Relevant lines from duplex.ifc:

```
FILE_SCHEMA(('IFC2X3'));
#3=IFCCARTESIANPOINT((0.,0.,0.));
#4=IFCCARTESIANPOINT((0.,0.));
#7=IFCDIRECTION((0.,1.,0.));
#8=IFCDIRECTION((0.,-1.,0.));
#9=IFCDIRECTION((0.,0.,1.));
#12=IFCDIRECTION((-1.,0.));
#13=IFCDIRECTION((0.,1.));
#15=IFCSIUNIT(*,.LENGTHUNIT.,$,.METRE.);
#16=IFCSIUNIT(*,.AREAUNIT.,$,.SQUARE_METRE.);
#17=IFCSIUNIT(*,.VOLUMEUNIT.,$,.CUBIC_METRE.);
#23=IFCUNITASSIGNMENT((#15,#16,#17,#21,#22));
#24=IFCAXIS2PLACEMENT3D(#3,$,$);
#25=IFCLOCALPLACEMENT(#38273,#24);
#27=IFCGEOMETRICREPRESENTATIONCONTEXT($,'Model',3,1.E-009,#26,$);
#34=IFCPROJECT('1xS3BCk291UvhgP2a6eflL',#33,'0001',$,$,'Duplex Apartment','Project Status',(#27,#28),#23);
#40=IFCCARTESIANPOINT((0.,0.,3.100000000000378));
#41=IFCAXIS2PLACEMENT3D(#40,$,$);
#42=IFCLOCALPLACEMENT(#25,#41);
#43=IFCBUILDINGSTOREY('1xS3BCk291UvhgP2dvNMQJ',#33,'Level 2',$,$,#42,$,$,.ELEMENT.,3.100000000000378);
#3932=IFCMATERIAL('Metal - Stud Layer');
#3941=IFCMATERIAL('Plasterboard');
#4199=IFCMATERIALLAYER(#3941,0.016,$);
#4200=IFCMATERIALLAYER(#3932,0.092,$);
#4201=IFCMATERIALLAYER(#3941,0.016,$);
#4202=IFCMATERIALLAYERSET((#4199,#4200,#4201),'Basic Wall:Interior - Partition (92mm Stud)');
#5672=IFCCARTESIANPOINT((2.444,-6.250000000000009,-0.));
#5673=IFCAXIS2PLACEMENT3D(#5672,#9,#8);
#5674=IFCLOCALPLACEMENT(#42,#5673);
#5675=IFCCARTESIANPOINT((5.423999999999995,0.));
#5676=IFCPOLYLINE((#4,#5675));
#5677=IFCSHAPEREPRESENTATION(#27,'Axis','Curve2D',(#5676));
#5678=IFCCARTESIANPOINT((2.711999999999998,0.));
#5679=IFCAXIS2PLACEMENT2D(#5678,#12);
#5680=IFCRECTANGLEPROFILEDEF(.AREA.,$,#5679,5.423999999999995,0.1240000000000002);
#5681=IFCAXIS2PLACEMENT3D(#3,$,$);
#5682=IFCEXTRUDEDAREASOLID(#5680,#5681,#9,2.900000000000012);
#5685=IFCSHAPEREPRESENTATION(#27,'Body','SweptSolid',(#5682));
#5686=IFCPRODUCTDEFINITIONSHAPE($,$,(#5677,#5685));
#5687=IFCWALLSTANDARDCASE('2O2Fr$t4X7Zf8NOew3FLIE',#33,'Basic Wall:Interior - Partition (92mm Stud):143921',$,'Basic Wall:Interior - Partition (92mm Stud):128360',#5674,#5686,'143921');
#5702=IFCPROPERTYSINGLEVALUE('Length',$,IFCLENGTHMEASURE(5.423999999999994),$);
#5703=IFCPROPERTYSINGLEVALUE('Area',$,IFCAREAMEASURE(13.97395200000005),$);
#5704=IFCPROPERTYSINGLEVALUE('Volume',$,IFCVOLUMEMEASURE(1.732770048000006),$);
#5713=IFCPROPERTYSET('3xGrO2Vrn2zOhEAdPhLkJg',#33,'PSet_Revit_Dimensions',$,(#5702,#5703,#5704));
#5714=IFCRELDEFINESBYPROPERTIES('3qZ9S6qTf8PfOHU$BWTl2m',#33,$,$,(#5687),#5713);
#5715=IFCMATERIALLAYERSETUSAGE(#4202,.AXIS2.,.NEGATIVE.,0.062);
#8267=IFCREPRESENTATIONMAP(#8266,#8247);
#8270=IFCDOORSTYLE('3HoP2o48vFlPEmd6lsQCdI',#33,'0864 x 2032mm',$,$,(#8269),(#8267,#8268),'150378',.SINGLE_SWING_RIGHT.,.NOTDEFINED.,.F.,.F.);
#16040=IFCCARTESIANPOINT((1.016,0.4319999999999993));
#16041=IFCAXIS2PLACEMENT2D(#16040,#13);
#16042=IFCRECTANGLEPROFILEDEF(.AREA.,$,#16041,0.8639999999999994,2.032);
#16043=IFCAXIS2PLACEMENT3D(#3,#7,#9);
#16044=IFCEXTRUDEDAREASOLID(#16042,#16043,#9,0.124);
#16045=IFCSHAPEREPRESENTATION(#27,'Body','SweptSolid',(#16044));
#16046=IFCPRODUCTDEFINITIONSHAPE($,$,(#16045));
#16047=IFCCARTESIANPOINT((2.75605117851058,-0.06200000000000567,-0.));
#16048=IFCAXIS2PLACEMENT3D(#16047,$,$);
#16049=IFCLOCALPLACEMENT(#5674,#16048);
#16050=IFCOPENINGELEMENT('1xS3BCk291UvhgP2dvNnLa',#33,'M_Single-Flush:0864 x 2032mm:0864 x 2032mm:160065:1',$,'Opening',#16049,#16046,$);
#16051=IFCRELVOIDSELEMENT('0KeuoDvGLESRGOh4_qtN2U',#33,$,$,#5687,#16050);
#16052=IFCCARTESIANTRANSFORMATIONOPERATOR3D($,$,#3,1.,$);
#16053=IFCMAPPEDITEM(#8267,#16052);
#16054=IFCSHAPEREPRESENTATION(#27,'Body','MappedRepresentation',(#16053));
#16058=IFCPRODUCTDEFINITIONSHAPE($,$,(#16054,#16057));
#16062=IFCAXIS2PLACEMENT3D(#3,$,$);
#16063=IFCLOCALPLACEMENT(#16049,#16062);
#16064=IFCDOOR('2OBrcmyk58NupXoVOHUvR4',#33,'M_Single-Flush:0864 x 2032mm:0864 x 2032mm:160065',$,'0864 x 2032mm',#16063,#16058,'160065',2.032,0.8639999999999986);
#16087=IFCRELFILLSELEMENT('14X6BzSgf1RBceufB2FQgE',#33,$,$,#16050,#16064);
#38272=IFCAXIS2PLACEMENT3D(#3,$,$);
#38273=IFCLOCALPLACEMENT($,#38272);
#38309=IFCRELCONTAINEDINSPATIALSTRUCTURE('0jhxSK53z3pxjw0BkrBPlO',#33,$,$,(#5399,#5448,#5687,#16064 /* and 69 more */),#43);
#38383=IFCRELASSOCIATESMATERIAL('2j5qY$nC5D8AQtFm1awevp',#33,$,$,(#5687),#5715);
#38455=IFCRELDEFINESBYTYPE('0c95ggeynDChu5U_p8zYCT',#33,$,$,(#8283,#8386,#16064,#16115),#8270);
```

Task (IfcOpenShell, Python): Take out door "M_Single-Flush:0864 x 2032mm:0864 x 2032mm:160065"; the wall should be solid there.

```python
import ifcopenshell
import ifcopenshell.api.feature
import ifcopenshell.api.pset
import ifcopenshell.api.root
import ifcopenshell.geom
import ifcopenshell.util.element
import ifcopenshell.util.shape
import ifcopenshell.util.unit

model = ifcopenshell.open("duplex.ifc")
area_scale = ifcopenshell.util.unit.calculate_unit_scale(model, "AREAUNIT")
volume_scale = ifcopenshell.util.unit.calculate_unit_scale(model, "VOLUMEUNIT")
settings = ifcopenshell.geom.settings()


def volume(element):
    """Net volume in cubic metres, openings subtracted."""
    shape = ifcopenshell.geom.create_shape(settings, element)
    return ifcopenshell.util.shape.get_volume(shape.geometry)


door = model.by_guid("2OBrcmyk58NupXoVOHUvR4")
opening = door.FillsVoids[0].RelatingOpeningElement
wall = opening.VoidsElements[0].RelatingBuildingElement
before = volume(wall)

ifcopenshell.api.root.remove_product(model, product=door)
ifcopenshell.api.feature.remove_feature(model, feature=opening)

after = volume(wall)
thickness = 0.124  # wall thickness in metres

# Update the wall's stored quantities.
pset = model.by_id(ifcopenshell.util.element.get_pset(wall, "PSet_Revit_Dimensions", should_inherit=False)["id"])
ifcopenshell.api.pset.edit_pset(model, pset=pset, properties={
    "Area": model.create_entity("IfcAreaMeasure", after / thickness / area_scale),
    "Volume": model.create_entity("IfcVolumeMeasure", after / volume_scale),
})

print(f"wall volume {before:.3f} -> {after:.3f} m3")

model.write("duplex_edited.ifc")
```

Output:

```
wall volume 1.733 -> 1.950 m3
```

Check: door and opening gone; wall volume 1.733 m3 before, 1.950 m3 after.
